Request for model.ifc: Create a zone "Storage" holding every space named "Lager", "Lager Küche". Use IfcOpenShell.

First a look at what the model holds.

```python
import ifcopenshell

model = ifcopenshell.open("model.ifc")
print(model.schema)
seen = {}
for space in model.by_type("IfcSpace"):
    seen[space.LongName] = seen.get(space.LongName, 0) + 1
for name, count in sorted(seen.items(), key=str):
    print(count, "x", name)
print("zones:", [z.Name for z in model.by_type("IfcZone")][:20])
```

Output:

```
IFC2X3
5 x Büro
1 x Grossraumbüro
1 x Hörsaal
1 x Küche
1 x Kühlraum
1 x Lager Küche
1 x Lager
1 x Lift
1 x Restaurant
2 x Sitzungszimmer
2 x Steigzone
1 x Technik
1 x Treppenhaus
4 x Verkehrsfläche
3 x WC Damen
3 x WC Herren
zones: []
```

```python
import ifcopenshell
import ifcopenshell.api.group
import ifcopenshell.api.root

model = ifcopenshell.open("model.ifc")

names = {"Lager", "Lager Küche"}
spaces = [s for s in model.by_type("IfcSpace") if s.LongName in names]

zone = ifcopenshell.api.root.create_entity(model, ifc_class="IfcZone", name="Storage")
ifcopenshell.api.group.assign_group(model, products=spaces, group=zone)
print(len(spaces), "spaces in", zone.Name)

model.write("model_rev.ifc")
```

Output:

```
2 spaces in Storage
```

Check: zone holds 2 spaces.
